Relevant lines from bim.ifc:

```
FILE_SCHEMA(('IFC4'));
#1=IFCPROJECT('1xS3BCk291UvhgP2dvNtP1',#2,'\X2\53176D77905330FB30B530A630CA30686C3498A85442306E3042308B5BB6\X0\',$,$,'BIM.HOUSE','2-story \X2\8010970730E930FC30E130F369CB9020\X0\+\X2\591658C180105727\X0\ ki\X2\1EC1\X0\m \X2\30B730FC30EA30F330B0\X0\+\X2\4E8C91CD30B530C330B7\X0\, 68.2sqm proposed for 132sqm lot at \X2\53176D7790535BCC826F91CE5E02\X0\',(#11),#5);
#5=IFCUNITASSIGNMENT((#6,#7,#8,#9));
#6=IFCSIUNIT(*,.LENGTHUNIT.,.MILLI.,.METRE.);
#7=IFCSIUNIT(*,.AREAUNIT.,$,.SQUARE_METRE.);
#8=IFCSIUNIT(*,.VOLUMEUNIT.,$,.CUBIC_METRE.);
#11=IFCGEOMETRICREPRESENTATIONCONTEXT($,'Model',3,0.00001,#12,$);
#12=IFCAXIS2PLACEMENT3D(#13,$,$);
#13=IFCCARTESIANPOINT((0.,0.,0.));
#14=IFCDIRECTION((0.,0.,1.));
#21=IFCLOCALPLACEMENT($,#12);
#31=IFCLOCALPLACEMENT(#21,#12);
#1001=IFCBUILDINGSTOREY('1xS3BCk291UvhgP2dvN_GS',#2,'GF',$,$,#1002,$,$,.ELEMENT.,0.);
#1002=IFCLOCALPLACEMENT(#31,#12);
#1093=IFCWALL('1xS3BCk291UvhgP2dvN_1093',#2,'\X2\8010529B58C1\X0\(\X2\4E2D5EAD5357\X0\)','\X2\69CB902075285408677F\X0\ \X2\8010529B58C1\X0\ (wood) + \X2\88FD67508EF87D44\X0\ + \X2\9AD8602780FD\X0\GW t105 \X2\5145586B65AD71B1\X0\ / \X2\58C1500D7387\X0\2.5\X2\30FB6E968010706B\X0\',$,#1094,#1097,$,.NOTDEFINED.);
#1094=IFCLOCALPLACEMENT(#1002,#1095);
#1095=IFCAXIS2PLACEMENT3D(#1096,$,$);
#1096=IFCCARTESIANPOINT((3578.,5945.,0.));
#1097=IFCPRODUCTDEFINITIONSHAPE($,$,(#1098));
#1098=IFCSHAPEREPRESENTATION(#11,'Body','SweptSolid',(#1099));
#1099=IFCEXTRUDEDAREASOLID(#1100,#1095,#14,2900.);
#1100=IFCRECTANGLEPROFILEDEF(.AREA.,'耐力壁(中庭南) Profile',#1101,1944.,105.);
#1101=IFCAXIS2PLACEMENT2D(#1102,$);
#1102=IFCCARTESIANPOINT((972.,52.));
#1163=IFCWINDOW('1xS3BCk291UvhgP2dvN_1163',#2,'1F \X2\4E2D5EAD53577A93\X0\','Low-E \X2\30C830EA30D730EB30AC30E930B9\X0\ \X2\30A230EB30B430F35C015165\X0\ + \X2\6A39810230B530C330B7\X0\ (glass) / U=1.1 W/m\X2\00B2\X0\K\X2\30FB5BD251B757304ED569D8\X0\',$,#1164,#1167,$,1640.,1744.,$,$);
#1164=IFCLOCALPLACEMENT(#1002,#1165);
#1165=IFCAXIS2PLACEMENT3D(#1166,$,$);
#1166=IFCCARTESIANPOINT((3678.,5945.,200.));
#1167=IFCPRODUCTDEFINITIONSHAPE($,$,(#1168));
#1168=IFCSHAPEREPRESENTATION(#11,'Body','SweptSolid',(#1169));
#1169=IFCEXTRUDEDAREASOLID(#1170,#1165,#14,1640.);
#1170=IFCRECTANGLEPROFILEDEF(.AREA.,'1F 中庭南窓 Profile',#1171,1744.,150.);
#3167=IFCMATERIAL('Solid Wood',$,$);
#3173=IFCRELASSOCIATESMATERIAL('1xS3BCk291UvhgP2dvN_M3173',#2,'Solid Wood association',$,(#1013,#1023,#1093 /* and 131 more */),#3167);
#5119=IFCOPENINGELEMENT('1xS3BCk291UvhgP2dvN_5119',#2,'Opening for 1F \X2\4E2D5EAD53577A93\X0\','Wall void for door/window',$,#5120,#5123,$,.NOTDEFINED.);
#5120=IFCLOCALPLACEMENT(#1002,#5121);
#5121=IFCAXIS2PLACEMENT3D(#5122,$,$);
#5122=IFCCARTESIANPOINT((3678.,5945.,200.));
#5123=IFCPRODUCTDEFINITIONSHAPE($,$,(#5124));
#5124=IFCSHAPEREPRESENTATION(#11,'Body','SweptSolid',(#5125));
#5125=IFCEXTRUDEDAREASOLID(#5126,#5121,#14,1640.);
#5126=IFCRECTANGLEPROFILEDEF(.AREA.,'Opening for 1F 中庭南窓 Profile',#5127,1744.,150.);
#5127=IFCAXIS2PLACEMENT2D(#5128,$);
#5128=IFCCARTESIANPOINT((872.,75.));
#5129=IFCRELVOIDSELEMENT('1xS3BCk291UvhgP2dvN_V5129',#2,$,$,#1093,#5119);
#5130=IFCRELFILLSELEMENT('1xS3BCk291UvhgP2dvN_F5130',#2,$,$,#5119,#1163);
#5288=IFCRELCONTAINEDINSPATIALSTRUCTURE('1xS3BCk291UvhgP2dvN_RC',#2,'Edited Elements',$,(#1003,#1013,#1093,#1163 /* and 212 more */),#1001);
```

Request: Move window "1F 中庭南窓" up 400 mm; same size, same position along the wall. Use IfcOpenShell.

```python
import numpy as np
import ifcopenshell
import ifcopenshell.api.geometry
import ifcopenshell.util.placement
import ifcopenshell.util.unit

model = ifcopenshell.open("bim.ifc")
unit_scale = ifcopenshell.util.unit.calculate_unit_scale(model)

window = model.by_guid("1xS3BCk291UvhgP2dvN_1163")
opening = window.FillsVoids[0].RelatingOpeningElement
dz = 0.4 / unit_scale

shift = np.array([0.0, 0.0, dz])
# The window is not placed relative to its opening, so move both.
for product in (opening, window):
    matrix = ifcopenshell.util.placement.get_local_placement(product.ObjectPlacement)
    matrix[:3, 3] += shift
    ifcopenshell.api.geometry.edit_object_placement(model, product=product, matrix=matrix, is_si=False)

print(f"moved by {dz * unit_scale:+.3f} m")

model.write("bim_rev.ifc")
```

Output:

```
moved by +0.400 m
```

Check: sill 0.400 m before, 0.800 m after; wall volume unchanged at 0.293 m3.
